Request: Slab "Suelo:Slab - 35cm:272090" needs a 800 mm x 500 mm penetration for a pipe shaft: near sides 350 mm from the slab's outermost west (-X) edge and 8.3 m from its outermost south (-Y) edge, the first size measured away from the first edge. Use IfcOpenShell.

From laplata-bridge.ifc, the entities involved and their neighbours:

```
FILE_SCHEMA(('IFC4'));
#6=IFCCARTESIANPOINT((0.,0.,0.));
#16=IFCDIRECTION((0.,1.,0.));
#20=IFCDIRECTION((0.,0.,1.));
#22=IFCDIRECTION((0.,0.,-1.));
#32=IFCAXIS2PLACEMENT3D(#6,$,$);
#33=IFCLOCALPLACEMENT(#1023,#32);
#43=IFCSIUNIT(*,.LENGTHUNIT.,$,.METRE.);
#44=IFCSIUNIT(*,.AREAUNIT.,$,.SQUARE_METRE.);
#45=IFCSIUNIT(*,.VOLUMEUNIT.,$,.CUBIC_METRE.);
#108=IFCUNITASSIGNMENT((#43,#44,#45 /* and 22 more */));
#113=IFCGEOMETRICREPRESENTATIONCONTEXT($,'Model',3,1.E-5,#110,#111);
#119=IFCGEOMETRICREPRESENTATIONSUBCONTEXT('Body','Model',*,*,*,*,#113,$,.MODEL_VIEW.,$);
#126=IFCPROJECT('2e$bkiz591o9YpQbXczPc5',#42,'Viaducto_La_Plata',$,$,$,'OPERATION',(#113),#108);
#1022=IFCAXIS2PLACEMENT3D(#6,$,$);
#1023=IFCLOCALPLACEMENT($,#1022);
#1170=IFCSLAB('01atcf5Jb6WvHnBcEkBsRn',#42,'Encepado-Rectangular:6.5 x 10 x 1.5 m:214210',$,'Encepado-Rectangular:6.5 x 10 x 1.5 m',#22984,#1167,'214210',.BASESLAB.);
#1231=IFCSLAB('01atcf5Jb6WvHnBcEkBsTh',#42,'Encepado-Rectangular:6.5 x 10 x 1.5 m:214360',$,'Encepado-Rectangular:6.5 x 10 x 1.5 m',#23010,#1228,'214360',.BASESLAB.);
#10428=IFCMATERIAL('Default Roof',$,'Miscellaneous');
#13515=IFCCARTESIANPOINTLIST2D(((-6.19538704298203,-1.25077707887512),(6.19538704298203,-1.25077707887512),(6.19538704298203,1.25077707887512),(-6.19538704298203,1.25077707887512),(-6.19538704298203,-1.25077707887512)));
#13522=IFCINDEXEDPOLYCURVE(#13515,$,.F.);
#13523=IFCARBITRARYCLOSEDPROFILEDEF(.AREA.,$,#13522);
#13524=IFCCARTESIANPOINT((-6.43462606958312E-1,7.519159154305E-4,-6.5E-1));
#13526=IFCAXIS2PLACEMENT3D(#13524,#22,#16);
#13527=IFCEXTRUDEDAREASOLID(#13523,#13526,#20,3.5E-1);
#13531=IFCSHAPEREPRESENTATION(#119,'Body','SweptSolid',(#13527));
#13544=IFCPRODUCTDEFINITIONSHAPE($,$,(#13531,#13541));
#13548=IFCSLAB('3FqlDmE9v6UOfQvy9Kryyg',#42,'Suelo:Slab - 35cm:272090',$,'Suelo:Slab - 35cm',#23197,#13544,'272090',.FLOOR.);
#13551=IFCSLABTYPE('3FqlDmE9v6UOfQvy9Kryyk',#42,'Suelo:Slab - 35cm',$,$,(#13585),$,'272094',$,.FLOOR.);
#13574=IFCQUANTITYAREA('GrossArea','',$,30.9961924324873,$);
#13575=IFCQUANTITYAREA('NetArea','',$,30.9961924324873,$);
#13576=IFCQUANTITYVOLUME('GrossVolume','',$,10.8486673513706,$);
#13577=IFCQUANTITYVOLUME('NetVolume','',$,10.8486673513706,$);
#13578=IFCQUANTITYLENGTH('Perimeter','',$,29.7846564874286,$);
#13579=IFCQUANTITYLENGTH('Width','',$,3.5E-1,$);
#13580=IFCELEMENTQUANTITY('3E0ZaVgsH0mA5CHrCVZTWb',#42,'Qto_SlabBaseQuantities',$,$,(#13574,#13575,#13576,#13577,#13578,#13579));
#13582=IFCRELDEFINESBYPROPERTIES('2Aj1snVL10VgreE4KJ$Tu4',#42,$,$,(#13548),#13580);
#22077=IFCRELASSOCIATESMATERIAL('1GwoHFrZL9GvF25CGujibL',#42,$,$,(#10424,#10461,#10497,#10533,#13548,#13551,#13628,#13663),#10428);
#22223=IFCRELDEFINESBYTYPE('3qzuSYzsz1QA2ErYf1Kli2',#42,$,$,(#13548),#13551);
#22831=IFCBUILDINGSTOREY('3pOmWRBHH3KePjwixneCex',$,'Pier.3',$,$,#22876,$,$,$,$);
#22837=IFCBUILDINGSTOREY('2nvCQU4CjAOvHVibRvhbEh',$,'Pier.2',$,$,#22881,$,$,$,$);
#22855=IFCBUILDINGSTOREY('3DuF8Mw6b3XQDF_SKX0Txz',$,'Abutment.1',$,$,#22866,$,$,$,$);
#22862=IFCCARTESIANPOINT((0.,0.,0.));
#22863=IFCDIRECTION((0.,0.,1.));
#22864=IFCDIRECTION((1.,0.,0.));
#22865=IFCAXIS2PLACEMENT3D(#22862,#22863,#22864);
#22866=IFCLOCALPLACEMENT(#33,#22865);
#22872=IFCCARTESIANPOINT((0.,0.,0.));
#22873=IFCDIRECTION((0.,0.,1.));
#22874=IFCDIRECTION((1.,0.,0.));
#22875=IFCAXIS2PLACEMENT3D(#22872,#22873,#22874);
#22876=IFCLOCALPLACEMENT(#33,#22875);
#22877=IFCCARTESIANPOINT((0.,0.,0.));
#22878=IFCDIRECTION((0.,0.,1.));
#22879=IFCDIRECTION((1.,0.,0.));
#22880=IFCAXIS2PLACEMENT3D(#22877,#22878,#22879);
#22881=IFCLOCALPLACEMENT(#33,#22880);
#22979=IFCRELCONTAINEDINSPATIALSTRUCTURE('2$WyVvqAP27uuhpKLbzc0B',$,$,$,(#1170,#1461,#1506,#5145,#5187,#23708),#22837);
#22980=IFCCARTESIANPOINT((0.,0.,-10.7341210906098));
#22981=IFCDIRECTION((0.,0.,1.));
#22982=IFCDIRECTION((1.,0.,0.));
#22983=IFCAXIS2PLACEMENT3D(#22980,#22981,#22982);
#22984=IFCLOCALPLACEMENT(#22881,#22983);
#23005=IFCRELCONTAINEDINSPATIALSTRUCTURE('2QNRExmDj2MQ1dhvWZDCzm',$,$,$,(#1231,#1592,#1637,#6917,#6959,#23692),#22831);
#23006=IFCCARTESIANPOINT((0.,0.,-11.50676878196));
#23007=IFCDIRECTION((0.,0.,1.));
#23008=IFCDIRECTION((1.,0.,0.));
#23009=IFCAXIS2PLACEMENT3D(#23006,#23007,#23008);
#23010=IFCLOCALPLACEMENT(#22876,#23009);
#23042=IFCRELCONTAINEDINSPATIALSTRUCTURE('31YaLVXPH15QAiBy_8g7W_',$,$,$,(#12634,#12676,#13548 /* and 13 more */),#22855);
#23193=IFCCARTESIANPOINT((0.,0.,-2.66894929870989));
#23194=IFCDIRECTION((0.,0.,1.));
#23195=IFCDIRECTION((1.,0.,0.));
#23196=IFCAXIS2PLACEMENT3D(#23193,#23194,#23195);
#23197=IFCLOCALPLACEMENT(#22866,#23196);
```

```python
import numpy as np
import ifcopenshell
import ifcopenshell.api.feature
import ifcopenshell.api.geometry
import ifcopenshell.api.pset
import ifcopenshell.api.root
import ifcopenshell.geom
import ifcopenshell.util.element
import ifcopenshell.util.placement
import ifcopenshell.util.representation
import ifcopenshell.util.shape
import ifcopenshell.util.unit

model = ifcopenshell.open("laplata-bridge.ifc")
unit_scale = ifcopenshell.util.unit.calculate_unit_scale(model)
area_scale = ifcopenshell.util.unit.calculate_unit_scale(model, "AREAUNIT")
volume_scale = ifcopenshell.util.unit.calculate_unit_scale(model, "VOLUMEUNIT")
settings = ifcopenshell.geom.settings()


def volume(element):
    """Net volume in cubic metres, openings subtracted."""
    shape = ifcopenshell.geom.create_shape(settings, element)
    return ifcopenshell.util.shape.get_volume(shape.geometry)


slab = model.by_guid("3FqlDmE9v6UOfQvy9Kryyg")
before = volume(slab)

# Extent in the slab's own axes, in metres. The edges named are its -X and -Y sides.
slab_shape = ifcopenshell.geom.create_shape(settings, slab)
vertices = ifcopenshell.util.shape.get_vertices(slab_shape.geometry)
x_min, y_min, bottom = vertices.min(axis=0)
top = vertices[:, 2].max()

opening = ifcopenshell.api.root.create_entity(model, ifc_class="IfcOpeningElement", name="Pipe shaft opening", predefined_type="OPENING")
context = ifcopenshell.util.representation.get_context(model, "Model", "Body", "MODEL_VIEW")
width, depth = 0.8, 0.5
outline = [(0.0, 0.0), (width, 0.0), (width, depth), (0.0, depth), (0.0, 0.0)]
# Overshoot both faces by 50 mm so the cut is clean.
shape = ifcopenshell.api.geometry.add_slab_representation(
    model, context=context, depth=top - bottom + 0.1, polyline=outline
)
ifcopenshell.api.geometry.assign_representation(model, product=opening, representation=shape)

matrix = ifcopenshell.util.placement.get_local_placement(slab.ObjectPlacement)
matrix[:, 3] = matrix @ np.append(np.array([x_min + 0.35, y_min + 8.3, bottom - 0.05]) / unit_scale, 1.0)
ifcopenshell.api.geometry.edit_object_placement(model, product=opening, matrix=matrix, is_si=False)
ifcopenshell.api.feature.add_feature(model, feature=opening, element=slab)

after = volume(slab)

# Update the slab's stored quantities.
qto = model.by_id(ifcopenshell.util.element.get_pset(slab, "Qto_SlabBaseQuantities", should_inherit=False)["id"])
ifcopenshell.api.pset.edit_qto(model, qto=qto, properties={
    "NetArea": after / (top - bottom) / area_scale,
    "NetVolume": after / volume_scale,
})

print(f"slab volume {before:.3f} -> {after:.3f} m3")

model.write("laplata-bridge_updated.ifc")
```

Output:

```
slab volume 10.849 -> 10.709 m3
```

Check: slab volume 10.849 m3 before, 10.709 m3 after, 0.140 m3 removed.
